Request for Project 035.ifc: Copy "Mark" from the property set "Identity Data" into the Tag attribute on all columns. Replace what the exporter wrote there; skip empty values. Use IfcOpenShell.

First a look at what the model holds.

```python
import ifcopenshell
import ifcopenshell.util.element

model = ifcopenshell.open("Project 035.ifc")
print(model.schema)
columns = model.by_type("IfcColumn")
print(len(columns), "columns")
for e in columns[:8]:
    source = ifcopenshell.util.element.get_pset(e, "Identity Data", "Mark")
    target = e.Tag
    print(e.id(), repr(source), repr(target), sep=" | ")
```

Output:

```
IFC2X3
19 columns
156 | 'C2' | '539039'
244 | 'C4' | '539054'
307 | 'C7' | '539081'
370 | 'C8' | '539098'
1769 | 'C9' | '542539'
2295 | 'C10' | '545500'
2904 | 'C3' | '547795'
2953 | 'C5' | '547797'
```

```python
import ifcopenshell
import ifcopenshell.util.element

model = ifcopenshell.open("Project 035.ifc")

count = 0
for e in model.by_type("IfcColumn"):
    value = ifcopenshell.util.element.get_pset(e, "Identity Data", "Mark")
    current = e.Tag
    if not value or not value.strip() or current == value:
        continue
    e.Tag = value
    count += 1

print(count, "columns updated")

model.write("Project 035_updated.ifc")
```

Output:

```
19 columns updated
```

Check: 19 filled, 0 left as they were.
